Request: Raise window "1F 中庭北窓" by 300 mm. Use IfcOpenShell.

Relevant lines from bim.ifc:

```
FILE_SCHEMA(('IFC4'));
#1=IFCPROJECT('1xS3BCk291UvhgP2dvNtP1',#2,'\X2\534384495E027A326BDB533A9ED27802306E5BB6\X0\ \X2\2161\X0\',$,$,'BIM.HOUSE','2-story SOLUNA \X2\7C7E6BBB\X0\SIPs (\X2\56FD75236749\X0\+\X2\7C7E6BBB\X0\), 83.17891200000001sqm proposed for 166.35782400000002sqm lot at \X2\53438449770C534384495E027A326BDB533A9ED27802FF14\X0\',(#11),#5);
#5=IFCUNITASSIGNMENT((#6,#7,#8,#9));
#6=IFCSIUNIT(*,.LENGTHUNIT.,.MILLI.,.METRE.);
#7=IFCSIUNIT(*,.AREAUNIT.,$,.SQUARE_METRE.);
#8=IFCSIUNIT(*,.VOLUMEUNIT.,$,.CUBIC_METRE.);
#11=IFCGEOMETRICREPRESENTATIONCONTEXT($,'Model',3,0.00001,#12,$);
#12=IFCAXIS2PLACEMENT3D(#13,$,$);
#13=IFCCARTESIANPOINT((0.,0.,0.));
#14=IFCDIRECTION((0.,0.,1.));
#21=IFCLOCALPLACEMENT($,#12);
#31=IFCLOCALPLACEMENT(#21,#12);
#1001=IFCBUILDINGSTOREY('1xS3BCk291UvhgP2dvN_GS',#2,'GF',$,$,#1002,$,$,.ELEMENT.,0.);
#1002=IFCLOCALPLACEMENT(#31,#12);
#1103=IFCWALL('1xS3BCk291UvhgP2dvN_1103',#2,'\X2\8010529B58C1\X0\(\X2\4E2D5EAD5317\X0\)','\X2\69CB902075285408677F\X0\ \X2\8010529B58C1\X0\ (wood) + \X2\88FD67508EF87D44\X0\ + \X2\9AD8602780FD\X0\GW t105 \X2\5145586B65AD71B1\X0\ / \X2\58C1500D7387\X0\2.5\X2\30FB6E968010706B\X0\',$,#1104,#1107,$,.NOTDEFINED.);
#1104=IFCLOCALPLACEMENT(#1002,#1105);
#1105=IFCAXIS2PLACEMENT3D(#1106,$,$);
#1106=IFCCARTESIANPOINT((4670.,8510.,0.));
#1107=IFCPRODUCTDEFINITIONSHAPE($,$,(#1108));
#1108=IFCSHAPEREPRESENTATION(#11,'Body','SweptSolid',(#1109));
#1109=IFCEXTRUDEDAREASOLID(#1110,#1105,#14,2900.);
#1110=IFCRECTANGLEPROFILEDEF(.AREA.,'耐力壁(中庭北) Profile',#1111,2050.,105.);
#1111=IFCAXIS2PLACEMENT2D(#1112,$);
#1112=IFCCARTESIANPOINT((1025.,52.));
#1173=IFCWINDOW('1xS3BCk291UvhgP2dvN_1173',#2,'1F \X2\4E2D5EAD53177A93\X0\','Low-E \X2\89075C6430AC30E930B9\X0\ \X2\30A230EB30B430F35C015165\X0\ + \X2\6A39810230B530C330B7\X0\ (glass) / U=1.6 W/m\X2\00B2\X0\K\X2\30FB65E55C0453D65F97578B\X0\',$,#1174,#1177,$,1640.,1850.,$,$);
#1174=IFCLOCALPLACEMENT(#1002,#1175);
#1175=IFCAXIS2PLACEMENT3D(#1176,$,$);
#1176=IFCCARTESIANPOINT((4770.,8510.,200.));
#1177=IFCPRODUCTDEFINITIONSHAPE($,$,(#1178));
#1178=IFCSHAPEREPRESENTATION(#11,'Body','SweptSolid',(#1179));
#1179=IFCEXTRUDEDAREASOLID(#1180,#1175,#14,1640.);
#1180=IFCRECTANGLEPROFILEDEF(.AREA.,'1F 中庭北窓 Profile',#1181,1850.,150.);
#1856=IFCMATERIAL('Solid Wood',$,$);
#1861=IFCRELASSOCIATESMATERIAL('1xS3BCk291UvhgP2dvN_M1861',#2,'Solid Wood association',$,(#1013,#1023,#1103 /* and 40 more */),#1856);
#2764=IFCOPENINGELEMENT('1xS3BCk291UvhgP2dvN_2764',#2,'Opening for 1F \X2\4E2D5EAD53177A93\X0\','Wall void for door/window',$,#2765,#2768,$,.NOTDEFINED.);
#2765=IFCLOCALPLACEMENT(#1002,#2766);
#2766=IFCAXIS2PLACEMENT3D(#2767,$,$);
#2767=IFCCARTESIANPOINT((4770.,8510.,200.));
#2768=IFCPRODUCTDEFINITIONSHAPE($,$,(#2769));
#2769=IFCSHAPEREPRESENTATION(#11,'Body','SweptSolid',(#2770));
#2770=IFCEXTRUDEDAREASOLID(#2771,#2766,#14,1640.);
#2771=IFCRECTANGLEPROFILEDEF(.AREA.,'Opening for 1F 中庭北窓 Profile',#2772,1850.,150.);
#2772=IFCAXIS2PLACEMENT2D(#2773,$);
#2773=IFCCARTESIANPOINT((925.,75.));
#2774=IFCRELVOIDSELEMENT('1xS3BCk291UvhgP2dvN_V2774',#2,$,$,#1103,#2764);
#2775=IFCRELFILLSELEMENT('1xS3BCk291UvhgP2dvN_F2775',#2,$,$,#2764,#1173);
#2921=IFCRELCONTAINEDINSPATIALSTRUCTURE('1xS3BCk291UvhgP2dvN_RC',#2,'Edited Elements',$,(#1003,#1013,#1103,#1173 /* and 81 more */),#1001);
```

```python
import numpy as np
import ifcopenshell
import ifcopenshell.api.geometry
import ifcopenshell.util.placement
import ifcopenshell.util.unit

model = ifcopenshell.open("bim.ifc")
unit_scale = ifcopenshell.util.unit.calculate_unit_scale(model)

window = model.by_id(1173)
opening = window.FillsVoids[0].RelatingOpeningElement
dz = 0.3 / unit_scale

shift = np.array([0.0, 0.0, dz])
# The window is not placed relative to its opening, so move both.
for product in (opening, window):
    matrix = ifcopenshell.util.placement.get_local_placement(product.ObjectPlacement)
    matrix[:3, 3] += shift
    ifcopenshell.api.geometry.edit_object_placement(model, product=product, matrix=matrix, is_si=False)

print(f"moved by {dz * unit_scale:+.3f} m")

model.write("bim_v2.ifc")
```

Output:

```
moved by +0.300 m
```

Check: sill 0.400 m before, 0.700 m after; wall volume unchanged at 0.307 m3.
